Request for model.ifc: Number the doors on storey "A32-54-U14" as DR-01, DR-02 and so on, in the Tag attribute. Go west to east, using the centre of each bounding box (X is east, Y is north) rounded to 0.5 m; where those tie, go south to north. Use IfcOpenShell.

First a look at what the model holds.

```python
import ifcopenshell
import ifcopenshell.util.element
import ifcopenshell.util.placement

model = ifcopenshell.open("model.ifc")
print(model.schema)
storey = next(s for s in model.by_type("IfcBuildingStorey") if s.Name == "A32-54-U14")
doors = [e for e in ifcopenshell.util.element.get_decomposition(storey) if e.is_a("IfcDoor")]
for e in sorted(doors, key=lambda e: e.id()):
    origin = ifcopenshell.util.placement.get_local_placement(e.ObjectPlacement)[:3, 3]
    print(e.id(), e.Tag, e.Name, origin.round(2) + 0.0, sep=" | ")
```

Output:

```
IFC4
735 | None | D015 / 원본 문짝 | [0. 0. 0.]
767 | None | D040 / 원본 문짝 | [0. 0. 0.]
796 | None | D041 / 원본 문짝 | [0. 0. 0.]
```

```python
import ifcopenshell
import ifcopenshell.geom
import ifcopenshell.util.element
import ifcopenshell.util.shape

model = ifcopenshell.open("model.ifc")
settings = ifcopenshell.geom.settings()
settings.set("use-world-coords", True)


def centre(element):
    shape = ifcopenshell.geom.create_shape(settings, element)
    return ifcopenshell.util.shape.get_bbox_centroid(shape.geometry)


storey = next(s for s in model.by_type("IfcBuildingStorey") if s.Name == "A32-54-U14")
doors = [e for e in ifcopenshell.util.element.get_decomposition(storey) if e.is_a("IfcDoor")]

# Insertion points can sit at a corner or the storey origin, so sort by the geometry (in metres).
centres = {e: centre(e) for e in doors}
doors.sort(key=lambda e: (round(centres[e][0] / 0.5), centres[e][1]))

for i, e in enumerate(doors, start=1):
    number = f"DR-{i:02d}"
    e.Tag = number
    print(e.id(), number)

model.write("model_updated.ifc")
```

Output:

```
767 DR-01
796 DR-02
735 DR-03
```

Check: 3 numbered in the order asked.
